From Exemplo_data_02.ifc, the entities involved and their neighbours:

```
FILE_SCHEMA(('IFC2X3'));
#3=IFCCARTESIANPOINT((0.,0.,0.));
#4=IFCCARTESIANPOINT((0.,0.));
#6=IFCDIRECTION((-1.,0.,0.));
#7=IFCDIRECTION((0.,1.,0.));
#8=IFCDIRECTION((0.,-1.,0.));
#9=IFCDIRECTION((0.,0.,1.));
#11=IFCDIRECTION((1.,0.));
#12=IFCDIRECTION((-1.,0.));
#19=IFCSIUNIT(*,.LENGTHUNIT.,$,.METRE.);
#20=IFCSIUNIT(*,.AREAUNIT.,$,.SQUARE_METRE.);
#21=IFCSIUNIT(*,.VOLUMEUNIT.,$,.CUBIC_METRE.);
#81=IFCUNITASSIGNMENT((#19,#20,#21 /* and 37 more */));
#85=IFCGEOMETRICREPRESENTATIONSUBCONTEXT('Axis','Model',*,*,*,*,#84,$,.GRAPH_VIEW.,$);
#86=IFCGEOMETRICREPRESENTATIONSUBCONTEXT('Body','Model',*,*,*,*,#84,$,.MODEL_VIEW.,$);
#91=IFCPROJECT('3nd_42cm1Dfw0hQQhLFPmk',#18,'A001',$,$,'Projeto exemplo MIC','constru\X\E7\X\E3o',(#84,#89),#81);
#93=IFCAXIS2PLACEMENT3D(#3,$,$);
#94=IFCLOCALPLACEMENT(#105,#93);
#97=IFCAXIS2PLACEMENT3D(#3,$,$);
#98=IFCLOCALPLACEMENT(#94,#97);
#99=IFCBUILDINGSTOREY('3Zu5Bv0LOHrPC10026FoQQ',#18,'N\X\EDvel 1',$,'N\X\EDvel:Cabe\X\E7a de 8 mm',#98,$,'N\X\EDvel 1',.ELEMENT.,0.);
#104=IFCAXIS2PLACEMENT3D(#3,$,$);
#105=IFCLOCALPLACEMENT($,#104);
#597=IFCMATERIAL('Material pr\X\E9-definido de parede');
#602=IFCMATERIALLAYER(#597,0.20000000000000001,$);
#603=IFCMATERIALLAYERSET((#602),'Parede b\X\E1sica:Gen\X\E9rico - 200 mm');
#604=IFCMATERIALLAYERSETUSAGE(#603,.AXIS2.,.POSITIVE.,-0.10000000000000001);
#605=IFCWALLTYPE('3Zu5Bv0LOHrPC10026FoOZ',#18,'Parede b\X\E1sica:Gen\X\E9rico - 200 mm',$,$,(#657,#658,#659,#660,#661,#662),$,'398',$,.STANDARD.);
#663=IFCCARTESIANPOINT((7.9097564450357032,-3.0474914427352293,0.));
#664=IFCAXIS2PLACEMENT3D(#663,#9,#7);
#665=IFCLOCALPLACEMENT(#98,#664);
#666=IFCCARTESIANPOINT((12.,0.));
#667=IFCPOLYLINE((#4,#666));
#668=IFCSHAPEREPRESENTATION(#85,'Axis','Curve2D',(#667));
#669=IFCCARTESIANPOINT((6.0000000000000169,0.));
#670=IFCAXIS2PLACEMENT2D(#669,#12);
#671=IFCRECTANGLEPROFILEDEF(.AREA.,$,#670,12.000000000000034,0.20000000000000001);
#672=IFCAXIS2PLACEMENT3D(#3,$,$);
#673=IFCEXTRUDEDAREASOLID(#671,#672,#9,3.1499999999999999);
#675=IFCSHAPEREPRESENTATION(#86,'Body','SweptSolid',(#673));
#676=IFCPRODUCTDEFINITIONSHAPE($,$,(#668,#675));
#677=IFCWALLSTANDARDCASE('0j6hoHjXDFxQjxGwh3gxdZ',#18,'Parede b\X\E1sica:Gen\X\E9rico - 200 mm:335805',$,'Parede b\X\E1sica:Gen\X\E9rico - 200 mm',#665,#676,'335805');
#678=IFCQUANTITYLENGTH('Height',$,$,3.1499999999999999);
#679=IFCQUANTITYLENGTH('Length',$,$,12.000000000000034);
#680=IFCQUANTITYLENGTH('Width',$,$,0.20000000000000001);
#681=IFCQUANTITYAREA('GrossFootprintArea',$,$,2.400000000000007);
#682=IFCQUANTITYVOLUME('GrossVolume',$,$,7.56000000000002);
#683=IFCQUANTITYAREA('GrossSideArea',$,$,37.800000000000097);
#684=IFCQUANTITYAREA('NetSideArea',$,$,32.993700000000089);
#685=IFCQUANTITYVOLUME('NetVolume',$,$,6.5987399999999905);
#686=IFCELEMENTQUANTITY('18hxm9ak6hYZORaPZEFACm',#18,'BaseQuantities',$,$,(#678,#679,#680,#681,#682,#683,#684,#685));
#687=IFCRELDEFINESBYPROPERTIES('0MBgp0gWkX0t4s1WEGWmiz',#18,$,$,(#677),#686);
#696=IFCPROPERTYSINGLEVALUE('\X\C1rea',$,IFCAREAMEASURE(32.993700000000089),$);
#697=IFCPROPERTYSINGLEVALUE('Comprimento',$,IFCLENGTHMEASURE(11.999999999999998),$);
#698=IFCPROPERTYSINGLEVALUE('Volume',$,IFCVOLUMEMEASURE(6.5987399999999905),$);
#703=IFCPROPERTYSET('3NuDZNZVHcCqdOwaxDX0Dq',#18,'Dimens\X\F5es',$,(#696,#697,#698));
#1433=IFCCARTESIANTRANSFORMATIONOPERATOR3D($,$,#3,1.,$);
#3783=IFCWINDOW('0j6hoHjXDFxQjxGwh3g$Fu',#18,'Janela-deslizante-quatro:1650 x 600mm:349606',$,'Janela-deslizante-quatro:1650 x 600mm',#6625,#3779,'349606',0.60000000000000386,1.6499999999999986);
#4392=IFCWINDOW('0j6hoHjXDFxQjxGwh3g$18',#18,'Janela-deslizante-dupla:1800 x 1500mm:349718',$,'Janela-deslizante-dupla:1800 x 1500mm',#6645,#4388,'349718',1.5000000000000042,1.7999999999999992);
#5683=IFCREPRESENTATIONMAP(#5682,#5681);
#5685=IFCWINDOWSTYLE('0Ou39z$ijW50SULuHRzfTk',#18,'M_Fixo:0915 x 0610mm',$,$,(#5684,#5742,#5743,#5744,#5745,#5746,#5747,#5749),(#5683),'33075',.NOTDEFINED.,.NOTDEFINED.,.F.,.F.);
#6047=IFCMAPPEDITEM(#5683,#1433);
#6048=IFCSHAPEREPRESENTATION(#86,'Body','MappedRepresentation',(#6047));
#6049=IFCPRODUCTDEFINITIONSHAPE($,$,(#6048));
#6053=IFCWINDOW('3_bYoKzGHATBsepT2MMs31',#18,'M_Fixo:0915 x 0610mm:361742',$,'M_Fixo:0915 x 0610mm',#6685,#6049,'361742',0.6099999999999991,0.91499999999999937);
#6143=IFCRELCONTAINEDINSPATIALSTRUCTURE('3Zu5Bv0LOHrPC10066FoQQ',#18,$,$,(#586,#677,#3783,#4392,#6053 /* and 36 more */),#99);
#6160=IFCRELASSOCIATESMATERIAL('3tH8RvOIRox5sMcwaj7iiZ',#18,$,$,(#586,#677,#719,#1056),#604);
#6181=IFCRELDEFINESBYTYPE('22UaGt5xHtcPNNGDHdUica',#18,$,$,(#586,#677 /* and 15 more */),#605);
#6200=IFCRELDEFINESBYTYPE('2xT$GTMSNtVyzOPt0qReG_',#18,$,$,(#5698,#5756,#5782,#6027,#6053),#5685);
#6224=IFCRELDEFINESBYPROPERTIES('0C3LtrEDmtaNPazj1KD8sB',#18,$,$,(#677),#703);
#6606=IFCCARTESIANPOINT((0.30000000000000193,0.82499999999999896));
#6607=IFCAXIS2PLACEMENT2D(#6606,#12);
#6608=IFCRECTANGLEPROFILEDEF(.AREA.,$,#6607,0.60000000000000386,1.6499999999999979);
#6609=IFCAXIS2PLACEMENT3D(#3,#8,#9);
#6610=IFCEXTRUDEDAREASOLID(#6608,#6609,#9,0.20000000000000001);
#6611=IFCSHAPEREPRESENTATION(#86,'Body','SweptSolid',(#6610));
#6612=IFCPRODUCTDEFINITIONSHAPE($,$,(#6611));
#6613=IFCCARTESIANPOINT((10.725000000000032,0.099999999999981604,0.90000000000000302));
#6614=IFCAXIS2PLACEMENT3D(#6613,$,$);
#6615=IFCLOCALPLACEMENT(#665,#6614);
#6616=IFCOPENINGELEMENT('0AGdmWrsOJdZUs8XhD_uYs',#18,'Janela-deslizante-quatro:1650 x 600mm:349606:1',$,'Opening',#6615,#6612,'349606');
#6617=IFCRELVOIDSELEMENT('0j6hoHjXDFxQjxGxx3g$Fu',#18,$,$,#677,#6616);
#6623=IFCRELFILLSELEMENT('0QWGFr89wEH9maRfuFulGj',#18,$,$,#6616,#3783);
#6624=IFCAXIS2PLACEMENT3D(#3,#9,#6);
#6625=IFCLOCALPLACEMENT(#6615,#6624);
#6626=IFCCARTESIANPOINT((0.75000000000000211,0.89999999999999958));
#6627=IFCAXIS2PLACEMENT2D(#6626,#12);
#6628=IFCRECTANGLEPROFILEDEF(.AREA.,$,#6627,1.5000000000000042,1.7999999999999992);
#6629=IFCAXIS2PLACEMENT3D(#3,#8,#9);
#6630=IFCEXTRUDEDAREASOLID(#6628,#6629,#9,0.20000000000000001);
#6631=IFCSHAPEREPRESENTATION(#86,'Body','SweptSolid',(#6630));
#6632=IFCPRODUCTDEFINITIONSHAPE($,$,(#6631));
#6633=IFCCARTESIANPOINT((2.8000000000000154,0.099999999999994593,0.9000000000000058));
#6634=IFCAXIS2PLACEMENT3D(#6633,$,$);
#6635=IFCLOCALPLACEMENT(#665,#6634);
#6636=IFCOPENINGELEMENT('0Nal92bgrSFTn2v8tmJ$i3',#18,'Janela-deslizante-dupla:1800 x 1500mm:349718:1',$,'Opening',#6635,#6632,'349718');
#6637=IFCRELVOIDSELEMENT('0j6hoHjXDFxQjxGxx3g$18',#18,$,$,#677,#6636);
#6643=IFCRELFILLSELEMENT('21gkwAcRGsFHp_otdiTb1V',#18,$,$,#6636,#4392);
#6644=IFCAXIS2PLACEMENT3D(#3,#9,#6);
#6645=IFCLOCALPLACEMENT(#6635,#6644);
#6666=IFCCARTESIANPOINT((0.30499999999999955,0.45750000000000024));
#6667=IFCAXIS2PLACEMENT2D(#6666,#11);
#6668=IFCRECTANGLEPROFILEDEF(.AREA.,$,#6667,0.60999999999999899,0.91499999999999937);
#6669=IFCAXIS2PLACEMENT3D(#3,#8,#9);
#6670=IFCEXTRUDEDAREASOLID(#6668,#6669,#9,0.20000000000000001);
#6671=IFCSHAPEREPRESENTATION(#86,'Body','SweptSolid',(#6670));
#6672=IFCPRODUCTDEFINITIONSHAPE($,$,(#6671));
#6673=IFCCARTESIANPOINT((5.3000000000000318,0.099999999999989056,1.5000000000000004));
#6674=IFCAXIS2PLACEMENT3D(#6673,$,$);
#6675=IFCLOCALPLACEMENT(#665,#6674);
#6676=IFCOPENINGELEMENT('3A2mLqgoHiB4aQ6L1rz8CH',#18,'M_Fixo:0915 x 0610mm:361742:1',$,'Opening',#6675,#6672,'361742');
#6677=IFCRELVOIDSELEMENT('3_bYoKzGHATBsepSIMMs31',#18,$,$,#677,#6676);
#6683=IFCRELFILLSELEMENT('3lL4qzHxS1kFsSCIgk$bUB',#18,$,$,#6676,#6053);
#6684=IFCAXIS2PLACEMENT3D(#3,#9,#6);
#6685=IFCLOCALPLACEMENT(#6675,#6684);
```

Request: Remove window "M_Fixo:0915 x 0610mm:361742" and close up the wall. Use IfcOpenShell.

```python
import ifcopenshell
import ifcopenshell.api.feature
import ifcopenshell.api.pset
import ifcopenshell.api.root
import ifcopenshell.geom
import ifcopenshell.util.element
import ifcopenshell.util.shape
import ifcopenshell.util.unit

model = ifcopenshell.open("Exemplo_data_02.ifc")
area_scale = ifcopenshell.util.unit.calculate_unit_scale(model, "AREAUNIT")
volume_scale = ifcopenshell.util.unit.calculate_unit_scale(model, "VOLUMEUNIT")
settings = ifcopenshell.geom.settings()


def volume(element):
    """Net volume in cubic metres, openings subtracted."""
    shape = ifcopenshell.geom.create_shape(settings, element)
    return ifcopenshell.util.shape.get_volume(shape.geometry)


window = model.by_id(6053)
opening = window.FillsVoids[0].RelatingOpeningElement
wall = opening.VoidsElements[0].RelatingBuildingElement
before = volume(wall)

ifcopenshell.api.root.remove_product(model, product=window)
ifcopenshell.api.feature.remove_feature(model, feature=opening)

after = volume(wall)
thickness = 0.2  # wall thickness in metres

# Update the wall's stored quantities.
qto = model.by_id(ifcopenshell.util.element.get_pset(wall, "BaseQuantities", should_inherit=False)["id"])
ifcopenshell.api.pset.edit_qto(model, qto=qto, properties={
    "NetSideArea": after / thickness / area_scale,
    "NetVolume": after / volume_scale,
})
pset = model.by_id(ifcopenshell.util.element.get_pset(wall, "Dimensões", should_inherit=False)["id"])
ifcopenshell.api.pset.edit_pset(model, pset=pset, properties={
    "Área": model.create_entity("IfcAreaMeasure", after / thickness / area_scale),
    "Volume": model.create_entity("IfcVolumeMeasure", after / volume_scale),
})

print(f"wall volume {before:.3f} -> {after:.3f} m3")

model.write("Exemplo_data_02_v2.ifc")
```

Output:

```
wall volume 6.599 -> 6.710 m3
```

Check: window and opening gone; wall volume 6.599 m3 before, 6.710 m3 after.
